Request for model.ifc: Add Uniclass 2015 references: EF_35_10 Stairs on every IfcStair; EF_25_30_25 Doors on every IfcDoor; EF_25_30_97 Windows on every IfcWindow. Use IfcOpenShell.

First a look at what the model holds.

```python
import ifcopenshell

model = ifcopenshell.open("model.ifc")
print(model.schema)
print("classifications:", [c.Name for c in model.by_type("IfcClassification")])
for ifc_class in ("IfcDoor", "IfcRoof", "IfcStair", "IfcWall", "IfcWindow"):
    print(ifc_class, len(model.by_type(ifc_class)))
```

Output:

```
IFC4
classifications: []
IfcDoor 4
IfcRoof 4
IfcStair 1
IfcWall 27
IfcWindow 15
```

```python
import ifcopenshell
import ifcopenshell.api.classification

model = ifcopenshell.open("model.ifc")

system = ifcopenshell.api.classification.add_classification(model, classification="Uniclass 2015")

codes = {
    "IfcStair": ("EF_35_10", "Stairs"),
    "IfcDoor": ("EF_25_30_25", "Doors"),
    "IfcWindow": ("EF_25_30_97", "Windows"),
}
for ifc_class, (code, name) in codes.items():
    products = model.by_type(ifc_class)
    ifcopenshell.api.classification.add_reference(
        model, products=products, classification=system, identification=code, name=name
    )
    print(code, len(products))

model.write("model-out.ifc")
```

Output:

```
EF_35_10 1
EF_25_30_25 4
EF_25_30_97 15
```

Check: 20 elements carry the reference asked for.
